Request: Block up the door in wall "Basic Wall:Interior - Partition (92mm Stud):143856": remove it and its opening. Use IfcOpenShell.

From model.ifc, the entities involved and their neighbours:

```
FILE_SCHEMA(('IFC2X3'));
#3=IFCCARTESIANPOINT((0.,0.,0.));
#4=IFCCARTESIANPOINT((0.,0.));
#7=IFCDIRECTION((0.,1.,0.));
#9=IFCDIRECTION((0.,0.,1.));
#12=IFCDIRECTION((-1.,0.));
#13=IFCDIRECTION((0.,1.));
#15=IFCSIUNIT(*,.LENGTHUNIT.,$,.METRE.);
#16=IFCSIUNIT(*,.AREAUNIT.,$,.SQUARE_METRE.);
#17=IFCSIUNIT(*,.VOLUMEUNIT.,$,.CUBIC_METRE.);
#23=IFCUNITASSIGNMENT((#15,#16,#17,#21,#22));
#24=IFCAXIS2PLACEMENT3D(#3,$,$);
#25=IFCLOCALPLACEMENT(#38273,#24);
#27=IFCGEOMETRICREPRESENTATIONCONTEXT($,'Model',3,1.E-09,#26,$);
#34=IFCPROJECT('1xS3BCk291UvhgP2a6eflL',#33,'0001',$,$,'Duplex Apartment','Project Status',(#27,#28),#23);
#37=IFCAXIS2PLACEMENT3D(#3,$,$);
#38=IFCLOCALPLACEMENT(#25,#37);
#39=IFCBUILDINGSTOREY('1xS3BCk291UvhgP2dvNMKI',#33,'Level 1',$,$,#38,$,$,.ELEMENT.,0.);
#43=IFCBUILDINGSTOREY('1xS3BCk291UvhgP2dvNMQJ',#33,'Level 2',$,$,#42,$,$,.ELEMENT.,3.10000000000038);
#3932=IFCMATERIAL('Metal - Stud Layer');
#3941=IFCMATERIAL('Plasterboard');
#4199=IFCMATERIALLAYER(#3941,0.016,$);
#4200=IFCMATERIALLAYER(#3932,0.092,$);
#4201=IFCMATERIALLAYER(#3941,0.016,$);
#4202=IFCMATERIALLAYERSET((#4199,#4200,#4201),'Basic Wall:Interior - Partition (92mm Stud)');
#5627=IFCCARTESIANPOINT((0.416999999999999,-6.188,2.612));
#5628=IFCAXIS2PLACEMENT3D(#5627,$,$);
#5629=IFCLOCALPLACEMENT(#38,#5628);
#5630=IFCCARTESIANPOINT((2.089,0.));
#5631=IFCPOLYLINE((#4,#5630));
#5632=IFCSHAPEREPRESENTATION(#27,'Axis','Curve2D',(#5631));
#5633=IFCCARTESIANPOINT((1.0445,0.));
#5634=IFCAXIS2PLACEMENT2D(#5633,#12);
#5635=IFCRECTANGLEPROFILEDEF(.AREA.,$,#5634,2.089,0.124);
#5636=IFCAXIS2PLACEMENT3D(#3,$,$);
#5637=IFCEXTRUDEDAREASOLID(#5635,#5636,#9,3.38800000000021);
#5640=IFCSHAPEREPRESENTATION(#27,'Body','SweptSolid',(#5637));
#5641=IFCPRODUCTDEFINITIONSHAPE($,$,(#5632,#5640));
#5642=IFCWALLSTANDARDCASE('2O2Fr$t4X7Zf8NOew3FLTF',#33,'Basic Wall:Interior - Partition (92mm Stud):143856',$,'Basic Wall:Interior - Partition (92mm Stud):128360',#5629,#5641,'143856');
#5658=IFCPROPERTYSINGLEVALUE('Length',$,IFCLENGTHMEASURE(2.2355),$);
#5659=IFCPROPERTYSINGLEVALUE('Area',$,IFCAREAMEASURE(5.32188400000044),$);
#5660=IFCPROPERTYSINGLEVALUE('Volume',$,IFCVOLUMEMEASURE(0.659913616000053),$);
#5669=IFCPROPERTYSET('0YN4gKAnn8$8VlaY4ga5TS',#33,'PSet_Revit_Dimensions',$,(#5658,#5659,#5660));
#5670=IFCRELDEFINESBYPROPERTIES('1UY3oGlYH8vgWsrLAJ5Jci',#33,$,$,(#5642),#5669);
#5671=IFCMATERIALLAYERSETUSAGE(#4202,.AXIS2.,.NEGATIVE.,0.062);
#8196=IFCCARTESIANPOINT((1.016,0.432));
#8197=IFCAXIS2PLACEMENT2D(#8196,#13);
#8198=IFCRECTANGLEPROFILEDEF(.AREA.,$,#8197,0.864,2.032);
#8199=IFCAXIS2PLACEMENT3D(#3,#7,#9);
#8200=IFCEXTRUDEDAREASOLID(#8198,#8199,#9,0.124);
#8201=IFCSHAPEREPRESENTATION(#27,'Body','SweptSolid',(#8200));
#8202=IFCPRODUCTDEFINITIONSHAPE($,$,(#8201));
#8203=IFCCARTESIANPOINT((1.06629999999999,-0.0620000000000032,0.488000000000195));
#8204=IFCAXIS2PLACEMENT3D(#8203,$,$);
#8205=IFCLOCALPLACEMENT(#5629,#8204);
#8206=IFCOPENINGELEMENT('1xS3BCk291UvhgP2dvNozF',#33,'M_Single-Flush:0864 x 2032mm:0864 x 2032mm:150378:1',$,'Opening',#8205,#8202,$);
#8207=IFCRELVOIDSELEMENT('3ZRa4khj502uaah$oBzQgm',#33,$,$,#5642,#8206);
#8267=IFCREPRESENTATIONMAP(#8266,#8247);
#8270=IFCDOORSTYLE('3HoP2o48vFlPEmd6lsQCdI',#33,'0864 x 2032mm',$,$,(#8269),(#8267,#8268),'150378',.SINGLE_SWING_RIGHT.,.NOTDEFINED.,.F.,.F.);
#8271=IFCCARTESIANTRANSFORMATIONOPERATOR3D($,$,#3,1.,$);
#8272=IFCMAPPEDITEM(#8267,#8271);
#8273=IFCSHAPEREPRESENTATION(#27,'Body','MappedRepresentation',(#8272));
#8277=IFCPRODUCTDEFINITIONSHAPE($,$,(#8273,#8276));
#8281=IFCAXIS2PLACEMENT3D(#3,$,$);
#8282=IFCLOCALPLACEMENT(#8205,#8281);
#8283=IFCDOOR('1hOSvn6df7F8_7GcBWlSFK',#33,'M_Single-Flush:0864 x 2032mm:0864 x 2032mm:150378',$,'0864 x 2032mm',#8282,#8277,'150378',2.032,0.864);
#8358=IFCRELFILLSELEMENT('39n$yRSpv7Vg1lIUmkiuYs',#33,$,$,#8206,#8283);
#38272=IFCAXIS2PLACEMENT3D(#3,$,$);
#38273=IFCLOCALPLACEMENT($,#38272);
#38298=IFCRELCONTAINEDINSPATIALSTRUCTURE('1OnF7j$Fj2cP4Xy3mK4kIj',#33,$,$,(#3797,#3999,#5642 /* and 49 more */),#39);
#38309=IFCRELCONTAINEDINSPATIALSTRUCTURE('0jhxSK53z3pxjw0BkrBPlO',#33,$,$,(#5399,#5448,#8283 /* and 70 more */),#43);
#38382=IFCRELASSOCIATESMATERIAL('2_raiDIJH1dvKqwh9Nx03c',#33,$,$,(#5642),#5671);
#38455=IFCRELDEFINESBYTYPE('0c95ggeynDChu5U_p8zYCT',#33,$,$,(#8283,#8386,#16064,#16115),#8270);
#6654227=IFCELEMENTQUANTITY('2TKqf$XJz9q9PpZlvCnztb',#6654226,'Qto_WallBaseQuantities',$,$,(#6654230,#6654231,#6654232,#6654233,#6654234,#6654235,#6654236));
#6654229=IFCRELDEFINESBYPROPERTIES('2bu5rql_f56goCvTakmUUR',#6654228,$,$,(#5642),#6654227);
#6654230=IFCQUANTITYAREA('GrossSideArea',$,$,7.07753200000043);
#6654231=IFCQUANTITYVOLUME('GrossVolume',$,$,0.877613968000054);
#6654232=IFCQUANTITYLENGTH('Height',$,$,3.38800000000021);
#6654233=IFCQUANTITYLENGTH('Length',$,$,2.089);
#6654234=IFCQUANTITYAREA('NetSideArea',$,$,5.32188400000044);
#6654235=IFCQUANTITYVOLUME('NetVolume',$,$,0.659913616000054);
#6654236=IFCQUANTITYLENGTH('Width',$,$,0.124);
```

```python
import ifcopenshell
import ifcopenshell.api.feature
import ifcopenshell.api.pset
import ifcopenshell.api.root
import ifcopenshell.geom
import ifcopenshell.util.element
import ifcopenshell.util.shape
import ifcopenshell.util.unit

model = ifcopenshell.open("model.ifc")
area_scale = ifcopenshell.util.unit.calculate_unit_scale(model, "AREAUNIT")
volume_scale = ifcopenshell.util.unit.calculate_unit_scale(model, "VOLUMEUNIT")
settings = ifcopenshell.geom.settings()


def volume(element):
    """Net volume in cubic metres, openings subtracted."""
    shape = ifcopenshell.geom.create_shape(settings, element)
    return ifcopenshell.util.shape.get_volume(shape.geometry)


door = model.by_guid("1hOSvn6df7F8_7GcBWlSFK")
opening = door.FillsVoids[0].RelatingOpeningElement
wall = opening.VoidsElements[0].RelatingBuildingElement
before = volume(wall)

ifcopenshell.api.root.remove_product(model, product=door)
ifcopenshell.api.feature.remove_feature(model, feature=opening)

after = volume(wall)
thickness = 0.124  # wall thickness in metres

# Update the wall's stored quantities.
pset = model.by_id(ifcopenshell.util.element.get_pset(wall, "PSet_Revit_Dimensions", should_inherit=False)["id"])
ifcopenshell.api.pset.edit_pset(model, pset=pset, properties={
    "Area": model.create_entity("IfcAreaMeasure", after / thickness / area_scale),
    "Volume": model.create_entity("IfcVolumeMeasure", after / volume_scale),
})
qto = model.by_id(ifcopenshell.util.element.get_pset(wall, "Qto_WallBaseQuantities", should_inherit=False)["id"])
ifcopenshell.api.pset.edit_qto(model, qto=qto, properties={
    "NetSideArea": after / thickness / area_scale,
    "NetVolume": after / volume_scale,
})

print(f"wall volume {before:.3f} -> {after:.3f} m3")

model.write("model_v2.ifc")
```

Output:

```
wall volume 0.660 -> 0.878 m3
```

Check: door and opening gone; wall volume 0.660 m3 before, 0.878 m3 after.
